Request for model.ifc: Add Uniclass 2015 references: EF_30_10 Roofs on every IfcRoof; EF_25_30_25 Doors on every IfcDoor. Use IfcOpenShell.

First a look at what the model holds.

```python
import ifcopenshell

model = ifcopenshell.open("model.ifc")
print(model.schema)
print("classifications:", [c.Name for c in model.by_type("IfcClassification")])
for ifc_class in ("IfcDoor", "IfcRoof", "IfcStair", "IfcWall", "IfcWindow"):
    print(ifc_class, len(model.by_type(ifc_class)))
```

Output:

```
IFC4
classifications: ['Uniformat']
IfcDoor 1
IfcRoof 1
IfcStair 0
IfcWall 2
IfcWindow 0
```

```python
import ifcopenshell
import ifcopenshell.api.classification

model = ifcopenshell.open("model.ifc")

system = ifcopenshell.api.classification.add_classification(model, classification="Uniclass 2015")

codes = {
    "IfcRoof": ("EF_30_10", "Roofs"),
    "IfcDoor": ("EF_25_30_25", "Doors"),
}
for ifc_class, (code, name) in codes.items():
    products = model.by_type(ifc_class)
    ifcopenshell.api.classification.add_reference(
        model, products=products, classification=system, identification=code, name=name
    )
    print(code, len(products))

model.write("model_rev.ifc")
```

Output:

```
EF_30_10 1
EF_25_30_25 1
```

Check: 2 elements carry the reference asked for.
